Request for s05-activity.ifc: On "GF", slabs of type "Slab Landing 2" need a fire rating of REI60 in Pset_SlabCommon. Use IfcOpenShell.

First a look at what the model holds.

```python
import ifcopenshell
import ifcopenshell.util.element

model = ifcopenshell.open("s05-activity.ifc")
print(model.schema)
storey = next(s for s in model.by_type("IfcBuildingStorey") if s.Name == "GF")
slabs = [e for e in ifcopenshell.util.element.get_decomposition(storey) if e.is_a("IfcSlab")]
seen = {}
for e in slabs:
    element_type = ifcopenshell.util.element.get_type(e)
    key = (element_type.Name if element_type != e and element_type else None, ifcopenshell.util.element.get_pset(e, "Pset_SlabCommon", "FireRating"))
    seen[key] = seen.get(key, 0) + 1
for (name, value), count in sorted(seen.items(), key=str):
    print(count, "x", name, "|", value)
```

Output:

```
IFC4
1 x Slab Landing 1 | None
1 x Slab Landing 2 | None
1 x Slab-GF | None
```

```python
import ifcopenshell
import ifcopenshell.api.pset
import ifcopenshell.util.element

model = ifcopenshell.open("s05-activity.ifc")

storey = next(s for s in model.by_type("IfcBuildingStorey") if s.Name == "GF")
slabs = [e for e in ifcopenshell.util.element.get_decomposition(storey) if e.is_a("IfcSlab")]

count = 0
for e in slabs:
    element_type = ifcopenshell.util.element.get_type(e)
    if element_type in (None, e) or element_type.Name != "Slab Landing 2":
        continue
    # add_pset returns the element's existing set when there is one.
    pset = ifcopenshell.api.pset.add_pset(model, product=e, name="Pset_SlabCommon")
    ifcopenshell.api.pset.edit_pset(model, pset=pset, properties={"FireRating": "REI60"})
    count += 1

print(count, "slabs updated")

model.write("s05-activity_v2.ifc")
```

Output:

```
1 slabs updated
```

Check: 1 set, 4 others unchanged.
